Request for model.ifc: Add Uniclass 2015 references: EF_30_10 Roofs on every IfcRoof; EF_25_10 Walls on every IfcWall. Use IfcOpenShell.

First a look at what the model holds.

```python
import ifcopenshell

model = ifcopenshell.open("model.ifc")
print(model.schema)
print("classifications:", [c.Name for c in model.by_type("IfcClassification")])
for ifc_class in ("IfcDoor", "IfcRoof", "IfcStair", "IfcWall", "IfcWindow"):
    print(ifc_class, len(model.by_type(ifc_class)))
```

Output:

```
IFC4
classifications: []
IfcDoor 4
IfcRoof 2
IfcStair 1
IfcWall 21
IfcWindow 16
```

```python
import ifcopenshell
import ifcopenshell.api.classification

model = ifcopenshell.open("model.ifc")

system = ifcopenshell.api.classification.add_classification(model, classification="Uniclass 2015")

codes = {
    "IfcRoof": ("EF_30_10", "Roofs"),
    "IfcWall": ("EF_25_10", "Walls"),
}
for ifc_class, (code, name) in codes.items():
    products = model.by_type(ifc_class)
    ifcopenshell.api.classification.add_reference(
        model, products=products, classification=system, identification=code, name=name
    )
    print(code, len(products))

model.write("model_rev.ifc")
```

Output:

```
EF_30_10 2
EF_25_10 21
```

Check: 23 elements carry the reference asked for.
